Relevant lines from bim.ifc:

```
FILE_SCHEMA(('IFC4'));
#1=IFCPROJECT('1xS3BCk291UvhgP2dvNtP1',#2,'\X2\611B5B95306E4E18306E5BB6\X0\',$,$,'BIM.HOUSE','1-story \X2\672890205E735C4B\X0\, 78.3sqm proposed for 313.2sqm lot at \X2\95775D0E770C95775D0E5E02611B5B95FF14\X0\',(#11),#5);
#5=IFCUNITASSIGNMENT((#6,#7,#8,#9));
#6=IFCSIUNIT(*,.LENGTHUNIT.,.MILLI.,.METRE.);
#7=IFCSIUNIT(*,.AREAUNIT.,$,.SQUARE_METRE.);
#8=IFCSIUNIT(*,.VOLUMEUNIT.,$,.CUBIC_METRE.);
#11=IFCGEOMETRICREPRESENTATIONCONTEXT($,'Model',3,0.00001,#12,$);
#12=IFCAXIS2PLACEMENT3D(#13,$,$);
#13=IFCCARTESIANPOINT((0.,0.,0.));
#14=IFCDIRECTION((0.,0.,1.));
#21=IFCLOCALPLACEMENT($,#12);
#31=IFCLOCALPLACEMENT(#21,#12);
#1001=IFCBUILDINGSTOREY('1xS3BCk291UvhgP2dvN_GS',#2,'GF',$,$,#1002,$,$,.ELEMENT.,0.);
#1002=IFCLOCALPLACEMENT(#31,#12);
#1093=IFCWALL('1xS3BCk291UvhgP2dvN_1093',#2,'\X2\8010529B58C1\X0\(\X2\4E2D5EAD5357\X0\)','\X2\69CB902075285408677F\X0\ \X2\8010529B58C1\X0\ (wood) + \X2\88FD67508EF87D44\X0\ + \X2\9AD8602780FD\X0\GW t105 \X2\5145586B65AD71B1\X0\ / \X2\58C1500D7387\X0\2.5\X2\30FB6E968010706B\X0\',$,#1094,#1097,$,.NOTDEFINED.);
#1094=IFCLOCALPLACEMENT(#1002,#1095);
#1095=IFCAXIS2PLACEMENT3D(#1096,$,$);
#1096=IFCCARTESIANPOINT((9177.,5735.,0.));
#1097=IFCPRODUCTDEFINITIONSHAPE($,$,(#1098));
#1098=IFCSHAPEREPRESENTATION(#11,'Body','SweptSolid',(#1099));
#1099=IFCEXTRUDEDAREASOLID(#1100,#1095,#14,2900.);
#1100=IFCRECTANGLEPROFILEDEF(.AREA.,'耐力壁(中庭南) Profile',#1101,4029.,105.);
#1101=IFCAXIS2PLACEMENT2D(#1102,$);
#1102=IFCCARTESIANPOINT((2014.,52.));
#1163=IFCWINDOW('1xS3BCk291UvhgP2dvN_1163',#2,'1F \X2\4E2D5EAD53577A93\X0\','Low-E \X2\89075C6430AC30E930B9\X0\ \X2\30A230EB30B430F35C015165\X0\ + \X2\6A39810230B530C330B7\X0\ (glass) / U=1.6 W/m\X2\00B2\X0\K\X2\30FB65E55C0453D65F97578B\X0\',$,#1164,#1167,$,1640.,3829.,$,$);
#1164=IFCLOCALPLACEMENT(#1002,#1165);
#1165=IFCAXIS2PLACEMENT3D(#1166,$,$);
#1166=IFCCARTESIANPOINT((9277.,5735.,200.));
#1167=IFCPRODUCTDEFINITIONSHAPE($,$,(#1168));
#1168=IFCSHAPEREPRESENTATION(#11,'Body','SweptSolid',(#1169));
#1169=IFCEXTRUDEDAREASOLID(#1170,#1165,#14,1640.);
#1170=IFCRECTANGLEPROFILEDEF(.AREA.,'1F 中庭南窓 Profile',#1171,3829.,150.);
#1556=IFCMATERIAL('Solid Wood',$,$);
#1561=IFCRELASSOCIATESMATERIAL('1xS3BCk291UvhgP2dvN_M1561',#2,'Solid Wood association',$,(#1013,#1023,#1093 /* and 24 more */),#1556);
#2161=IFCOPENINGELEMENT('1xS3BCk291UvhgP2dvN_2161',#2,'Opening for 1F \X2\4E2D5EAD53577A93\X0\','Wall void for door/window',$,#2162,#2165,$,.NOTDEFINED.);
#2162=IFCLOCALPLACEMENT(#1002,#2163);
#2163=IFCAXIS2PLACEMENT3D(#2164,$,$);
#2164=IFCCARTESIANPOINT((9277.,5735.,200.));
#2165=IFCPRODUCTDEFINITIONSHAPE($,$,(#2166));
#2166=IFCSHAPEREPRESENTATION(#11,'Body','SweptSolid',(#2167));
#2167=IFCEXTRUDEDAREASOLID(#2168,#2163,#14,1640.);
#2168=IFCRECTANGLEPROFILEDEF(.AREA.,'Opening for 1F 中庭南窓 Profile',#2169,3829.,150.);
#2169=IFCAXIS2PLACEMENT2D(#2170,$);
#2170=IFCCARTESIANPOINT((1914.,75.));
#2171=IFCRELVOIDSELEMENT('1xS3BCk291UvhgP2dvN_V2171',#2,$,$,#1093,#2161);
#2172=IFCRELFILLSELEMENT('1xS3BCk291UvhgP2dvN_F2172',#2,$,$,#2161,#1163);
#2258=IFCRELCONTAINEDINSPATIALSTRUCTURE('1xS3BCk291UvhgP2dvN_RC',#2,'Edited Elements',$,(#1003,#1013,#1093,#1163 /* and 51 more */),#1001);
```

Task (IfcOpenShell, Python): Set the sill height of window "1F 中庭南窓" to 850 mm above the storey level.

```python
import numpy as np
import ifcopenshell
import ifcopenshell.api.geometry
import ifcopenshell.geom
import ifcopenshell.util.element
import ifcopenshell.util.placement
import ifcopenshell.util.shape
import ifcopenshell.util.unit

model = ifcopenshell.open("bim.ifc")
unit_scale = ifcopenshell.util.unit.calculate_unit_scale(model)

window = model.by_guid("1xS3BCk291UvhgP2dvN_1163")
opening = window.FillsVoids[0].RelatingOpeningElement
storey = ifcopenshell.util.element.get_container(window, ifc_class="IfcBuildingStorey")
level = ifcopenshell.util.placement.get_local_placement(storey.ObjectPlacement)[2, 3]

# The opening's origin need not be at the sill, so measure its lowest point.
shape = ifcopenshell.geom.create_shape(ifcopenshell.geom.settings(), opening)
bottom = ifcopenshell.util.shape.get_shape_bottom_elevation(shape, shape.geometry) / unit_scale
dz = level + 850.0 - bottom

shift = np.array([0.0, 0.0, dz])
# The window is not placed relative to its opening, so move both.
for product in (opening, window):
    matrix = ifcopenshell.util.placement.get_local_placement(product.ObjectPlacement)
    matrix[:3, 3] += shift
    ifcopenshell.api.geometry.edit_object_placement(model, product=product, matrix=matrix, is_si=False)

print(f"moved by {dz * unit_scale:+.3f} m")

model.write("bim_updated.ifc")
```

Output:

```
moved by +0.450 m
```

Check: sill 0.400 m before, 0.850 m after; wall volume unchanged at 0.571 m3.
